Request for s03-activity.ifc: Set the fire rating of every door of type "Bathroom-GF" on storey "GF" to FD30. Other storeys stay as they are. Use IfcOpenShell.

First a look at what the model holds.

```python
import ifcopenshell
import ifcopenshell.util.element

model = ifcopenshell.open("s03-activity.ifc")
print(model.schema)
storey = next(s for s in model.by_type("IfcBuildingStorey") if s.Name == "GF")
doors = [e for e in ifcopenshell.util.element.get_decomposition(storey) if e.is_a("IfcDoor")]
seen = {}
for e in doors:
    element_type = ifcopenshell.util.element.get_type(e)
    key = (element_type.Name if element_type != e and element_type else None, ifcopenshell.util.element.get_pset(e, "Pset_DoorCommon", "FireRating"))
    seen[key] = seen.get(key, 0) + 1
for (name, value), count in sorted(seen.items(), key=str):
    print(count, "x", name, "|", value)
```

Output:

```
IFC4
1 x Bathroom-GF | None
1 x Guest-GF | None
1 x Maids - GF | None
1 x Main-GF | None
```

```python
import ifcopenshell
import ifcopenshell.api.pset
import ifcopenshell.util.element

model = ifcopenshell.open("s03-activity.ifc")

storey = next(s for s in model.by_type("IfcBuildingStorey") if s.Name == "GF")
doors = [e for e in ifcopenshell.util.element.get_decomposition(storey) if e.is_a("IfcDoor")]

count = 0
for e in doors:
    element_type = ifcopenshell.util.element.get_type(e)
    if element_type in (None, e) or element_type.Name != "Bathroom-GF":
        continue
    # add_pset returns the element's existing set when there is one.
    pset = ifcopenshell.api.pset.add_pset(model, product=e, name="Pset_DoorCommon")
    ifcopenshell.api.pset.edit_pset(model, pset=pset, properties={"FireRating": "FD30"})
    count += 1

print(count, "doors updated")

model.write("s03-activity_v2.ifc")
```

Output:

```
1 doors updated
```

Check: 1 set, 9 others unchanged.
